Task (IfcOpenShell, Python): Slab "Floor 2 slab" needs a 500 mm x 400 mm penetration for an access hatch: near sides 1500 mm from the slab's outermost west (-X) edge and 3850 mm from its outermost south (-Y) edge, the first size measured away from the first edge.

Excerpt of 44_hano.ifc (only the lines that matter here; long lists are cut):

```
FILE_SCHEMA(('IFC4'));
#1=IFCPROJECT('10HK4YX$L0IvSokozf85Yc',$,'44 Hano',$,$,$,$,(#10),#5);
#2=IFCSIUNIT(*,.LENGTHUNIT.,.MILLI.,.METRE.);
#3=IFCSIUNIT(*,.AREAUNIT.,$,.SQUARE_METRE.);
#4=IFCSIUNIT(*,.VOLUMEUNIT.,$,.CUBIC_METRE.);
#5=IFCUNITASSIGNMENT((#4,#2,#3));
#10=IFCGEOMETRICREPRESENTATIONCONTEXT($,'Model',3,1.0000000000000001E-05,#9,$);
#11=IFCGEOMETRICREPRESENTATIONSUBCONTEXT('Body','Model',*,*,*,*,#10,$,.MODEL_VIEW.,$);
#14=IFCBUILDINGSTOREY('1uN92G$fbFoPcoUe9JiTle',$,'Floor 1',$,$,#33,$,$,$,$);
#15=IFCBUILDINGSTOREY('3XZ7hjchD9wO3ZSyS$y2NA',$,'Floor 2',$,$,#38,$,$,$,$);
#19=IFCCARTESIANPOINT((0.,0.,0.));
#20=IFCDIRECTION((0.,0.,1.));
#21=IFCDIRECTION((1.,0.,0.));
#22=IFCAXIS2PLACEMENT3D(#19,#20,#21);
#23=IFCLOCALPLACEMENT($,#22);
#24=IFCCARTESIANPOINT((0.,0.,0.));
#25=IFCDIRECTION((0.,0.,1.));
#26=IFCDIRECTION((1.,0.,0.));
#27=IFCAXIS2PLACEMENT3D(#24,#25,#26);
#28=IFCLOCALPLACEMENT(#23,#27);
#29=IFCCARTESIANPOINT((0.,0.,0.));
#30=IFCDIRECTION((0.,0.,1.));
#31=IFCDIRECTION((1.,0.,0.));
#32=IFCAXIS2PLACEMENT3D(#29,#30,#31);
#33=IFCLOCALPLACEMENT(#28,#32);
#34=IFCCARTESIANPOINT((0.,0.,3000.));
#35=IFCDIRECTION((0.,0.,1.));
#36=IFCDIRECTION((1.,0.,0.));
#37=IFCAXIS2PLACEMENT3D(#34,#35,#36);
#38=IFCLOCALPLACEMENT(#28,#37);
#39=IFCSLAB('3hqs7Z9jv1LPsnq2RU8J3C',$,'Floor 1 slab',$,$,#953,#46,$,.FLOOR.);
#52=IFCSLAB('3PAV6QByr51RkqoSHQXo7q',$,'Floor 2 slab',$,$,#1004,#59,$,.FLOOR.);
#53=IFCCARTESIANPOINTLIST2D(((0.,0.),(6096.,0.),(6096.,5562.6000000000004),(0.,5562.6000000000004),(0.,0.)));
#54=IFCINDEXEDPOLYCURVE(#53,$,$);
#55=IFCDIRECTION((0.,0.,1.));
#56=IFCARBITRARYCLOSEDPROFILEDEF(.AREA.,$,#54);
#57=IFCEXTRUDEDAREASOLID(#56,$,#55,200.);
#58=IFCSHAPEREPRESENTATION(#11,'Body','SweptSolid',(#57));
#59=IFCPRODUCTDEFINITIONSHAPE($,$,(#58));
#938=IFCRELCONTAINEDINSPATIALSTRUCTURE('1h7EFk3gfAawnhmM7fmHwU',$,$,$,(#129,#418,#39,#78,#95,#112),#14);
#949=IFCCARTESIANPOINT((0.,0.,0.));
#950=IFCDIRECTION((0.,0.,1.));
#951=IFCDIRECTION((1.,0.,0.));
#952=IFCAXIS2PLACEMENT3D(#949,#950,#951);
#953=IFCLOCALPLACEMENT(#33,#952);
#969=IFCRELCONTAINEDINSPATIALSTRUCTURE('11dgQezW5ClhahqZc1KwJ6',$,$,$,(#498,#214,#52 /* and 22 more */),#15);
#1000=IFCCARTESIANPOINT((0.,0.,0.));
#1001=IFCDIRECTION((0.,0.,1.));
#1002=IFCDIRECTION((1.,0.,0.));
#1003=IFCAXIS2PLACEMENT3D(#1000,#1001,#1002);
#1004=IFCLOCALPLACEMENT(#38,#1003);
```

```python
import numpy as np
import ifcopenshell
import ifcopenshell.api.feature
import ifcopenshell.api.geometry
import ifcopenshell.api.root
import ifcopenshell.geom
import ifcopenshell.util.placement
import ifcopenshell.util.representation
import ifcopenshell.util.shape
import ifcopenshell.util.unit

model = ifcopenshell.open("44_hano.ifc")
unit_scale = ifcopenshell.util.unit.calculate_unit_scale(model)
settings = ifcopenshell.geom.settings()


def volume(element):
    """Net volume in cubic metres, openings subtracted."""
    shape = ifcopenshell.geom.create_shape(settings, element)
    return ifcopenshell.util.shape.get_volume(shape.geometry)


slab = model.by_guid("3PAV6QByr51RkqoSHQXo7q")
before = volume(slab)

# Extent in the slab's own axes, in metres. The edges named are its -X and -Y sides.
slab_shape = ifcopenshell.geom.create_shape(settings, slab)
vertices = ifcopenshell.util.shape.get_vertices(slab_shape.geometry)
x_min, y_min, bottom = vertices.min(axis=0)
top = vertices[:, 2].max()

opening = ifcopenshell.api.root.create_entity(model, ifc_class="IfcOpeningElement", name="Access hatch opening", predefined_type="OPENING")
context = ifcopenshell.util.representation.get_context(model, "Model", "Body", "MODEL_VIEW")
width, depth = 0.5, 0.4
outline = [(0.0, 0.0), (width, 0.0), (width, depth), (0.0, depth), (0.0, 0.0)]
# Overshoot both faces by 50 mm so the cut is clean.
shape = ifcopenshell.api.geometry.add_slab_representation(
    model, context=context, depth=top - bottom + 0.1, polyline=outline
)
ifcopenshell.api.geometry.assign_representation(model, product=opening, representation=shape)

matrix = ifcopenshell.util.placement.get_local_placement(slab.ObjectPlacement)
matrix[:, 3] = matrix @ np.append(np.array([x_min + 1.5, y_min + 3.85, bottom - 0.05]) / unit_scale, 1.0)
ifcopenshell.api.geometry.edit_object_placement(model, product=opening, matrix=matrix, is_si=False)
ifcopenshell.api.feature.add_feature(model, feature=opening, element=slab)

after = volume(slab)

print(f"slab volume {before:.3f} -> {after:.3f} m3")

model.write("44_hano_edited.ifc")
```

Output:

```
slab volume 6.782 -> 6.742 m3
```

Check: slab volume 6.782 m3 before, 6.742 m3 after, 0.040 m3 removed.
